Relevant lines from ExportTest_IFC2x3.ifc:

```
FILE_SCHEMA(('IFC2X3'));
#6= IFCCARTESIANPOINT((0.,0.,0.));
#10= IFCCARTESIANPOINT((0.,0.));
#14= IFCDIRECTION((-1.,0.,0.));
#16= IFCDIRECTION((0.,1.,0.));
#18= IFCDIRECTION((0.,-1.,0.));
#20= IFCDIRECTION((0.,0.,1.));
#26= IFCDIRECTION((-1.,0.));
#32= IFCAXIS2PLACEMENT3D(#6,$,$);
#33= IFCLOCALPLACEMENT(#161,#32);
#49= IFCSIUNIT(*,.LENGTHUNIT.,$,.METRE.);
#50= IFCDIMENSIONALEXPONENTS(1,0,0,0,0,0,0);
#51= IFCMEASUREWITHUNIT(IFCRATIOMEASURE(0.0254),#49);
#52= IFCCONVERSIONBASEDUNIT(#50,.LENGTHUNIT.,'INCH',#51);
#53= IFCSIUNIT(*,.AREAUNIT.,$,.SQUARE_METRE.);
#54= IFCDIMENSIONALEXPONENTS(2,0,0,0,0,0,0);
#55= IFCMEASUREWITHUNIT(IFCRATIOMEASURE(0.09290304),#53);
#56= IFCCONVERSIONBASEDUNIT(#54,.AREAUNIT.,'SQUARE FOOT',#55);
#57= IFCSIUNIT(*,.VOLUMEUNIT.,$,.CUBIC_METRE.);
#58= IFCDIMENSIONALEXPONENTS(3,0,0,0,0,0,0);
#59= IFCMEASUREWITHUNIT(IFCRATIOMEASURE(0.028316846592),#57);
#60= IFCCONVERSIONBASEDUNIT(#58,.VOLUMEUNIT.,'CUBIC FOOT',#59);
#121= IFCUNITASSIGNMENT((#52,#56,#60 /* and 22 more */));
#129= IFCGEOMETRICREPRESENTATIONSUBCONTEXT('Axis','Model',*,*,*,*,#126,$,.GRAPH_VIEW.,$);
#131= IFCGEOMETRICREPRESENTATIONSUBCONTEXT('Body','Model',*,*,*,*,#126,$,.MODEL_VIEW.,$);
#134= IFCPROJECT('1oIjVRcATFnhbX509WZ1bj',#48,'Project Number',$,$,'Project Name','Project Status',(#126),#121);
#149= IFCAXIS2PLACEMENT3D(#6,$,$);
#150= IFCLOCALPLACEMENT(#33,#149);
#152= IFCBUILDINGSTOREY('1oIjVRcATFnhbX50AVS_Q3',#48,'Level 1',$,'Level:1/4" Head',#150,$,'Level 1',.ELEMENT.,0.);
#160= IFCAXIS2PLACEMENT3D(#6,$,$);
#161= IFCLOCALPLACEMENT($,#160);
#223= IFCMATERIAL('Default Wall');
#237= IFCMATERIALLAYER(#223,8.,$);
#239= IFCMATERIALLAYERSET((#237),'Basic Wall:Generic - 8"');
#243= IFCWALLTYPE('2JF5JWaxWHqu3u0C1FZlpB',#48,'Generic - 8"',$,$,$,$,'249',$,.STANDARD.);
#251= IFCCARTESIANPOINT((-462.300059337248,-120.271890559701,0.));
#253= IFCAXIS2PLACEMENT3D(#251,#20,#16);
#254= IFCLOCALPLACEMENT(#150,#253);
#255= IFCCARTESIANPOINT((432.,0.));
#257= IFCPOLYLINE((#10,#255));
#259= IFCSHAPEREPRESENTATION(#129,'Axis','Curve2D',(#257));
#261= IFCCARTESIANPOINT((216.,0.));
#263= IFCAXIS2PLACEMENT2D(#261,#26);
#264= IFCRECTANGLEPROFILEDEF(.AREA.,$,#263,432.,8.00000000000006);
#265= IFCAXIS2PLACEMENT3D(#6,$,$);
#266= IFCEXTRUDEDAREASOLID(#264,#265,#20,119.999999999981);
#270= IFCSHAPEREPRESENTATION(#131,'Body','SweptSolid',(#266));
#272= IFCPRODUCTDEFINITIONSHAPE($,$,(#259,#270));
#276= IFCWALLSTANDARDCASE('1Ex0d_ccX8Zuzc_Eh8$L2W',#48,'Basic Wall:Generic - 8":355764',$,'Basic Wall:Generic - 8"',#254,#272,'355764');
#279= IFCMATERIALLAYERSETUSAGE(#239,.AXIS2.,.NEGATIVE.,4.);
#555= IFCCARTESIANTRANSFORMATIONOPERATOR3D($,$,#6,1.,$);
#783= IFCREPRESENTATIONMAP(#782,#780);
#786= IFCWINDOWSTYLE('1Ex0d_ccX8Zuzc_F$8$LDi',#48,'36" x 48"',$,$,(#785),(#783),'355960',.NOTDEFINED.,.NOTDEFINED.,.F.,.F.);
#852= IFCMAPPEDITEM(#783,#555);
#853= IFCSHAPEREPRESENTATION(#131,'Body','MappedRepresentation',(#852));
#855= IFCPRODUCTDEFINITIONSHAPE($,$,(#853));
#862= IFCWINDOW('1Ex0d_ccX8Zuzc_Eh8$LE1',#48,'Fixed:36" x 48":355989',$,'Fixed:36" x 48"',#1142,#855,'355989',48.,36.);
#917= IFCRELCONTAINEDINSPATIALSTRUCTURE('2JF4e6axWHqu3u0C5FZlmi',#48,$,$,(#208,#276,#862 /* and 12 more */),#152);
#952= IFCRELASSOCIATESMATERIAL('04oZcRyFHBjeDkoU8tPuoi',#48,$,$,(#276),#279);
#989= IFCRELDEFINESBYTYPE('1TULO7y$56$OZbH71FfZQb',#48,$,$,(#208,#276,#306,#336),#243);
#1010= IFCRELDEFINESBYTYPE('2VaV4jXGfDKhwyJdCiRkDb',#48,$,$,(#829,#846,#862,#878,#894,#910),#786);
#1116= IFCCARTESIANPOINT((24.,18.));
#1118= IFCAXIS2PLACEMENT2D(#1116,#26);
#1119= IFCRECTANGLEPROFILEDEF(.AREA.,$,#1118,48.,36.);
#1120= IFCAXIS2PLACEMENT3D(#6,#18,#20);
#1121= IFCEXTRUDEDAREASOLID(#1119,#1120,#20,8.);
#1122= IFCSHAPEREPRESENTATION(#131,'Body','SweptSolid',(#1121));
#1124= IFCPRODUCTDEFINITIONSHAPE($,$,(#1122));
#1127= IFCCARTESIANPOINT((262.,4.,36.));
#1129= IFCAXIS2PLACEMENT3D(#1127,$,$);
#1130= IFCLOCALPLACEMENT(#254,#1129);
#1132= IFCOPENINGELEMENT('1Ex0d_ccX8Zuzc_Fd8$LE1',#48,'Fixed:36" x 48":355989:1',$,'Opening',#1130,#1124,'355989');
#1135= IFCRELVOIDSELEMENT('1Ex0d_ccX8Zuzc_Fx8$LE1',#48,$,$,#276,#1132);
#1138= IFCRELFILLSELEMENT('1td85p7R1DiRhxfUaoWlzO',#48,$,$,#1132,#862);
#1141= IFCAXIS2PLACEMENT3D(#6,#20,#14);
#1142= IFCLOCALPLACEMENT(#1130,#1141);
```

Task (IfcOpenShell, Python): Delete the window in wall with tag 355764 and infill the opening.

```python
import ifcopenshell
import ifcopenshell.api.feature
import ifcopenshell.api.root
import ifcopenshell.geom
import ifcopenshell.util.shape

model = ifcopenshell.open("ExportTest_IFC2x3.ifc")
settings = ifcopenshell.geom.settings()


def volume(element):
    """Net volume in cubic metres, openings subtracted."""
    shape = ifcopenshell.geom.create_shape(settings, element)
    return ifcopenshell.util.shape.get_volume(shape.geometry)


window = model.by_guid("1Ex0d_ccX8Zuzc_Eh8$LE1")
opening = window.FillsVoids[0].RelatingOpeningElement
wall = opening.VoidsElements[0].RelatingBuildingElement
before = volume(wall)

ifcopenshell.api.root.remove_product(model, product=window)
ifcopenshell.api.feature.remove_feature(model, feature=opening)

after = volume(wall)

print(f"wall volume {before:.3f} -> {after:.3f} m3")

model.write("ExportTest_IFC2x3-out.ifc")
```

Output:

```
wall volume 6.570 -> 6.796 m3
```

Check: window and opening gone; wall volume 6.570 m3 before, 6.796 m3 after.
